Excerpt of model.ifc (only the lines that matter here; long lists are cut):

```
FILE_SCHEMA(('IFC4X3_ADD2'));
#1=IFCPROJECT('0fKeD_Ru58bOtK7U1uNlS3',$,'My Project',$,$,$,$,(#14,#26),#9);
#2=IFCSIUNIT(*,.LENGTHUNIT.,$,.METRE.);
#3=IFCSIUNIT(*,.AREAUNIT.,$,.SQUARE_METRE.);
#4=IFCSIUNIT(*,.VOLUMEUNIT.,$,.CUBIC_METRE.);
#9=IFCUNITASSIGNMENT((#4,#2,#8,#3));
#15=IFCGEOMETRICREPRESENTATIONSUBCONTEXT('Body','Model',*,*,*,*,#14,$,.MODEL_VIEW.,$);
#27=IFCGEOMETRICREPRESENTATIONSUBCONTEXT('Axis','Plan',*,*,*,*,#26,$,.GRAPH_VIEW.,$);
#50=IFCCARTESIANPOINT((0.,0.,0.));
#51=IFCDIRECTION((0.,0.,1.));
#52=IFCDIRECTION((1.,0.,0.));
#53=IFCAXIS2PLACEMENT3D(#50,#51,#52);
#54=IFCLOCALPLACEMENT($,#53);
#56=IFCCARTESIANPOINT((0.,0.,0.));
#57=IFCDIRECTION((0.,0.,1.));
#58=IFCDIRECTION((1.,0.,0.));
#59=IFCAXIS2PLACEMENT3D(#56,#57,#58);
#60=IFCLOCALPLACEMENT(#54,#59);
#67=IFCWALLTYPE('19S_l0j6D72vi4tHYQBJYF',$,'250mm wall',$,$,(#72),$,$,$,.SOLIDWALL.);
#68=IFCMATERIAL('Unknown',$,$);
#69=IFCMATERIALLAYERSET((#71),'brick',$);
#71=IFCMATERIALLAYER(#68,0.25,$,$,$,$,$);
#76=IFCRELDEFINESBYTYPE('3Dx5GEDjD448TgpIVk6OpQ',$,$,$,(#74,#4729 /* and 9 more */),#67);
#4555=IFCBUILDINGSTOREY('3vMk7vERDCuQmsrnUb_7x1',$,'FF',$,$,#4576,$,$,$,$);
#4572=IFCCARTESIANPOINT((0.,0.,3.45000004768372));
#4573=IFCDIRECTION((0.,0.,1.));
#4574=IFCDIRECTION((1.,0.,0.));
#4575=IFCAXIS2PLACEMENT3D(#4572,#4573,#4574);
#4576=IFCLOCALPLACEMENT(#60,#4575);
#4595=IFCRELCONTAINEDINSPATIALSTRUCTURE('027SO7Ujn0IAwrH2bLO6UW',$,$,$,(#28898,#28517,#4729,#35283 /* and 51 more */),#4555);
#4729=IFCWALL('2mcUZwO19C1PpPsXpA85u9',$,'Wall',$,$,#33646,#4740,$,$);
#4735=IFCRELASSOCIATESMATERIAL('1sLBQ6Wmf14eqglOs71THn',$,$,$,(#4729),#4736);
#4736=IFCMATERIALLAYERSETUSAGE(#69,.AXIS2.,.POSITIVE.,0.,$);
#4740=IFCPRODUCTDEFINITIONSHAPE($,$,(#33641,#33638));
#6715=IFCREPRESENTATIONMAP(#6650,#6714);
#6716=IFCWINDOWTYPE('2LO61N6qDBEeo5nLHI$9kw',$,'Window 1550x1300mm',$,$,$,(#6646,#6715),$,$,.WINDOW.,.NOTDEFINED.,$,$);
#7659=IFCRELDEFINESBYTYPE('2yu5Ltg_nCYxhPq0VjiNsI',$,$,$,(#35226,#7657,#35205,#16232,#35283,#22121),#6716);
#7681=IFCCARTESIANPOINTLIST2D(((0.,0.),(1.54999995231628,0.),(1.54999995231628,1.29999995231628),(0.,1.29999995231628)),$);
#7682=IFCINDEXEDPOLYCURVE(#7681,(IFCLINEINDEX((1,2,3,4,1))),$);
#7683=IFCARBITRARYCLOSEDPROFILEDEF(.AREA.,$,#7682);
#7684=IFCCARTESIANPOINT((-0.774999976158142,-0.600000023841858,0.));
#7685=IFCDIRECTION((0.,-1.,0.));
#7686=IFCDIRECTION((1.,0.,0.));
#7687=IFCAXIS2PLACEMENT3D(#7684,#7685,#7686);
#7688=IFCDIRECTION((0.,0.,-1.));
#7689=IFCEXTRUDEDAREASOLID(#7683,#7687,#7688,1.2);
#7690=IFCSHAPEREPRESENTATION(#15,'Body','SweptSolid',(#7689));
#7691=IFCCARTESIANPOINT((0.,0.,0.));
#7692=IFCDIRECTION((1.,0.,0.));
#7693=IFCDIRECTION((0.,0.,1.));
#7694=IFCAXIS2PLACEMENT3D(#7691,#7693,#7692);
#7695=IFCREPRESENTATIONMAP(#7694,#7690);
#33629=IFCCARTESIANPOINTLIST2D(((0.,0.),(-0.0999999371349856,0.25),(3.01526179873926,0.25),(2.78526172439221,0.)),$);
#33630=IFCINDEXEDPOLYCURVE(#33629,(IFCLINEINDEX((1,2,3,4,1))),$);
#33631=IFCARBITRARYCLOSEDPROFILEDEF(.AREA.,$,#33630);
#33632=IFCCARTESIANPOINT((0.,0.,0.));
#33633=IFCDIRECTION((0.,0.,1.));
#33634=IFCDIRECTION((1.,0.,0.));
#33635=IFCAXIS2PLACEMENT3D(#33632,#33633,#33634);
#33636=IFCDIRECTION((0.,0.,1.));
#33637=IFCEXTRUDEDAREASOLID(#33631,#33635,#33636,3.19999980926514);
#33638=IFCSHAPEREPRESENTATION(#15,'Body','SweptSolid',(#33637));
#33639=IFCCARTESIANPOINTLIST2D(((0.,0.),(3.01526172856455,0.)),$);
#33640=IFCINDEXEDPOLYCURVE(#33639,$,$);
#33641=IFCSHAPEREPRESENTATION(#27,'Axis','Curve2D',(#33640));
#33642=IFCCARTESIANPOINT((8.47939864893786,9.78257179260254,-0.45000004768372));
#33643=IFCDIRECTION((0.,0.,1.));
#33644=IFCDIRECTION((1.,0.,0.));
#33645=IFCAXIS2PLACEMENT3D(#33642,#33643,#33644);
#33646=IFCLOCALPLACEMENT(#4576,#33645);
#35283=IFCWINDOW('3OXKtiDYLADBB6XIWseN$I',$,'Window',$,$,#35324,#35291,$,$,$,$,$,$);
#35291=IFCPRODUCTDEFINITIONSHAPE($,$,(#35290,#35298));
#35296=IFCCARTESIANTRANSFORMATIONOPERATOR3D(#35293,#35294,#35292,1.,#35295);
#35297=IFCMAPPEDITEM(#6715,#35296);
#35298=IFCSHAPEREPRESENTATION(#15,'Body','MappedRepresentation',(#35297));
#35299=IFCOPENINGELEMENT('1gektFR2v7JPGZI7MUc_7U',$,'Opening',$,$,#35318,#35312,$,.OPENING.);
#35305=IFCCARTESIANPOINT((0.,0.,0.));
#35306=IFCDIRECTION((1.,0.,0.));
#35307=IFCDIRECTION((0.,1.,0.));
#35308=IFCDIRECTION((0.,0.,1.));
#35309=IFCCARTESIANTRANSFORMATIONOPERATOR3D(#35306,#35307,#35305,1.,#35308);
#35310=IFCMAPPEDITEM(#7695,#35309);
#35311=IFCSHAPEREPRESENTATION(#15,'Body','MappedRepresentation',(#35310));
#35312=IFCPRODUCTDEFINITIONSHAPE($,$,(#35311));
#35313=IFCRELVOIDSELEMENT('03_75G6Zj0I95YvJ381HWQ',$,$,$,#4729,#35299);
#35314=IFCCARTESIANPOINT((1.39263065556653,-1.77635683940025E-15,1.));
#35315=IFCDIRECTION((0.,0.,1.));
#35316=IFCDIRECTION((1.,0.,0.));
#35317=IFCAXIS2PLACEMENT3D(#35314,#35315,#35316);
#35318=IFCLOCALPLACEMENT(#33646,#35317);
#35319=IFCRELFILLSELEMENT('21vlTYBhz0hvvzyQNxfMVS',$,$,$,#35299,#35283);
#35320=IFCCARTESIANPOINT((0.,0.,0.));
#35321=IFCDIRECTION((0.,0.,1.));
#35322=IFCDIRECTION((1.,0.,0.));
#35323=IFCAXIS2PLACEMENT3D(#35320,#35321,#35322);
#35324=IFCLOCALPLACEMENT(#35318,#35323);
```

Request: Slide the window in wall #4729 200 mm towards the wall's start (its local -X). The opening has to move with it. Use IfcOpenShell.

```python
import ifcopenshell
import ifcopenshell.api.geometry
import ifcopenshell.util.placement

model = ifcopenshell.open("model.ifc")

window = model.by_guid("3OXKtiDYLADBB6XIWseN$I")
opening = window.FillsVoids[0].RelatingOpeningElement
wall = opening.VoidsElements[0].RelatingBuildingElement

wall_matrix = ifcopenshell.util.placement.get_local_placement(wall.ObjectPlacement)
shift = wall_matrix[:3, 0] * -0.2
before = ifcopenshell.util.placement.get_local_placement(window.ObjectPlacement)[:3, 3].copy()

# The window is placed relative to its opening, so it follows when the opening moves.
matrix = ifcopenshell.util.placement.get_local_placement(opening.ObjectPlacement)
matrix[:3, 3] += shift
ifcopenshell.api.geometry.edit_object_placement(
    model, product=opening, matrix=matrix, is_si=False, should_transform_children=True
)

after = ifcopenshell.util.placement.get_local_placement(window.ObjectPlacement)[:3, 3]
print("window moved by", (after - before).round(3) + 0.0)

model.write("model_v2.ifc")
```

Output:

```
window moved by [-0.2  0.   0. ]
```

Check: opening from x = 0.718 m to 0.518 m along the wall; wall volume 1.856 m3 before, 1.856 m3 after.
